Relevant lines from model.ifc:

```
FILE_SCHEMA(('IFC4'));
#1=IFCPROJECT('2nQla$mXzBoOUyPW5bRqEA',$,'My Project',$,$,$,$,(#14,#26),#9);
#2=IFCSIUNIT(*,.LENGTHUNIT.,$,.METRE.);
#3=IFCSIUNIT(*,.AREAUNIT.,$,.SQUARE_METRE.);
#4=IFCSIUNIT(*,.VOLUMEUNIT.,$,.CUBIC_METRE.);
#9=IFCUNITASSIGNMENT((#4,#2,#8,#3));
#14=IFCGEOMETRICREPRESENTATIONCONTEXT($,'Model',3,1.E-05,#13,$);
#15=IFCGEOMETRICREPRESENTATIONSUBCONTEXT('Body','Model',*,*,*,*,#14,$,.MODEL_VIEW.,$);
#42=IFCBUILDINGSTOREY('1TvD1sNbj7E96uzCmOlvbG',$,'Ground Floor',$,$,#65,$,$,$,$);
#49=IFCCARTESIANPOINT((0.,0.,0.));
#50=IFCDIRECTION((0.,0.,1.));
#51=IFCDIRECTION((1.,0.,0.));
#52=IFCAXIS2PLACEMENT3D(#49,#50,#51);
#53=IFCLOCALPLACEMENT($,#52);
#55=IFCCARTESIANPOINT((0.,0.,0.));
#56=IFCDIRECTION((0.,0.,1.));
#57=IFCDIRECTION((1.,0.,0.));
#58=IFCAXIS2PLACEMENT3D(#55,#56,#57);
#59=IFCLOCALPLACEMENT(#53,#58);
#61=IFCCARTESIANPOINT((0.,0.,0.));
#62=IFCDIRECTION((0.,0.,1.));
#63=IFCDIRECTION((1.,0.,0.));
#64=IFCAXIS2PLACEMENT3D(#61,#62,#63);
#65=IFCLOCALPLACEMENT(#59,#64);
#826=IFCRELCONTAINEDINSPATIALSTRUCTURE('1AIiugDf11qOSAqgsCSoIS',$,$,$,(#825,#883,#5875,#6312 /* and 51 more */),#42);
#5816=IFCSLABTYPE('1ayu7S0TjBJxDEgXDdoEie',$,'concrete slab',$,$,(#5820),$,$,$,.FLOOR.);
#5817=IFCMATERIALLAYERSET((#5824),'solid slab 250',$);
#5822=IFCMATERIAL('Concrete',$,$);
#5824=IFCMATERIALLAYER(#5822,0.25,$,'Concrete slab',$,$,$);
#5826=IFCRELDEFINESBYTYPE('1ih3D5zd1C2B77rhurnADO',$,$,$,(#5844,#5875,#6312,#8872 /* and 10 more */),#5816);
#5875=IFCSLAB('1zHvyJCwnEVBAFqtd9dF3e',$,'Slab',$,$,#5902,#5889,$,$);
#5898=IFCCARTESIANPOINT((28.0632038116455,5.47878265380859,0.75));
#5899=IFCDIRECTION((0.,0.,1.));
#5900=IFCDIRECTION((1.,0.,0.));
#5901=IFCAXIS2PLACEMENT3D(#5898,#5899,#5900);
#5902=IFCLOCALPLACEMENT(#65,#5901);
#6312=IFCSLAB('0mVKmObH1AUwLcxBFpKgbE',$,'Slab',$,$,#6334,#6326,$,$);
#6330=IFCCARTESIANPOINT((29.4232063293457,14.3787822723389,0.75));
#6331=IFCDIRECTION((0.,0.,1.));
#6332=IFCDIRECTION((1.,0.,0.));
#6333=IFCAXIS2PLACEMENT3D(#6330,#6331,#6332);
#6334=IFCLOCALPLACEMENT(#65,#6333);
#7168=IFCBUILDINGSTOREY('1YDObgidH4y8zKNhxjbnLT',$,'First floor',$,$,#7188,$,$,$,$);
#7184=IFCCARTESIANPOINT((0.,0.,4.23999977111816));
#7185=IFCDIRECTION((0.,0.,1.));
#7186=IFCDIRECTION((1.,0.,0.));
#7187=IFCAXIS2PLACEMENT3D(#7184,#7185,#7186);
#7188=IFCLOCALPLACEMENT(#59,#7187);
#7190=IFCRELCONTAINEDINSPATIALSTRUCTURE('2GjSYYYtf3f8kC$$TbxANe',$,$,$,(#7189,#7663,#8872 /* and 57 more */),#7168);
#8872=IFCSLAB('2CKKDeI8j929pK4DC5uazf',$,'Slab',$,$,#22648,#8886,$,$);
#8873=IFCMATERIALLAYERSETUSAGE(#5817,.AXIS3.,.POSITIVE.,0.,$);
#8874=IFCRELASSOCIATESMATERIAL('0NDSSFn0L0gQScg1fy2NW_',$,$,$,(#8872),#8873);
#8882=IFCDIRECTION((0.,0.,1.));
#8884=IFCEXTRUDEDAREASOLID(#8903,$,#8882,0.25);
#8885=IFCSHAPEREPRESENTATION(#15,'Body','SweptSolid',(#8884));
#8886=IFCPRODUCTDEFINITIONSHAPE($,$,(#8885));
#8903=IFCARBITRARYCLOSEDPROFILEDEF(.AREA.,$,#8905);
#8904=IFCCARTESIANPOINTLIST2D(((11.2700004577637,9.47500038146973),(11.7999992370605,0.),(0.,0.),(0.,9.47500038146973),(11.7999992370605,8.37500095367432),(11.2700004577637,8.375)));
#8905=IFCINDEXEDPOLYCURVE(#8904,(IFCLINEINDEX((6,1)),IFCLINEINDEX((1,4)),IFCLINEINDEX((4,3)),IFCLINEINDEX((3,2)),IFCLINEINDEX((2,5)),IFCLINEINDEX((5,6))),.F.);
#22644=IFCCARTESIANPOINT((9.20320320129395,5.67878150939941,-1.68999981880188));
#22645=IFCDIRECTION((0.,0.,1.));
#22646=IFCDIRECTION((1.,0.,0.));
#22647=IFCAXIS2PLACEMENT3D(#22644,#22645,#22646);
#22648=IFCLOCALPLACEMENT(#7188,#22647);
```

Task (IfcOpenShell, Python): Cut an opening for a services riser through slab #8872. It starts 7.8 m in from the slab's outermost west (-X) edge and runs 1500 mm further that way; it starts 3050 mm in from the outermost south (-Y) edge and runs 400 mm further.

```python
import numpy as np
import ifcopenshell
import ifcopenshell.api.feature
import ifcopenshell.api.geometry
import ifcopenshell.api.root
import ifcopenshell.geom
import ifcopenshell.util.placement
import ifcopenshell.util.representation
import ifcopenshell.util.shape
import ifcopenshell.util.unit

model = ifcopenshell.open("model.ifc")
unit_scale = ifcopenshell.util.unit.calculate_unit_scale(model)
settings = ifcopenshell.geom.settings()


def volume(element):
    """Net volume in cubic metres, openings subtracted."""
    shape = ifcopenshell.geom.create_shape(settings, element)
    return ifcopenshell.util.shape.get_volume(shape.geometry)


slab = model.by_guid("2CKKDeI8j929pK4DC5uazf")
before = volume(slab)

# Extent in the slab's own axes, in metres. The edges named are its -X and -Y sides.
slab_shape = ifcopenshell.geom.create_shape(settings, slab)
vertices = ifcopenshell.util.shape.get_vertices(slab_shape.geometry)
x_min, y_min, bottom = vertices.min(axis=0)
top = vertices[:, 2].max()

opening = ifcopenshell.api.root.create_entity(model, ifc_class="IfcOpeningElement", name="Services riser opening", predefined_type="OPENING")
context = ifcopenshell.util.representation.get_context(model, "Model", "Body", "MODEL_VIEW")
width, depth = 1.5, 0.4
outline = [(0.0, 0.0), (width, 0.0), (width, depth), (0.0, depth), (0.0, 0.0)]
# Overshoot both faces by 50 mm so the cut is clean.
shape = ifcopenshell.api.geometry.add_slab_representation(
    model, context=context, depth=top - bottom + 0.1, polyline=outline
)
ifcopenshell.api.geometry.assign_representation(model, product=opening, representation=shape)

matrix = ifcopenshell.util.placement.get_local_placement(slab.ObjectPlacement)
matrix[:, 3] = matrix @ np.append(np.array([x_min + 7.8, y_min + 3.05, bottom - 0.05]) / unit_scale, 1.0)
ifcopenshell.api.geometry.edit_object_placement(model, product=opening, matrix=matrix, is_si=False)
ifcopenshell.api.feature.add_feature(model, feature=opening, element=slab)

after = volume(slab)

print(f"slab volume {before:.3f} -> {after:.3f} m3")

model.write("model_edited.ifc")
```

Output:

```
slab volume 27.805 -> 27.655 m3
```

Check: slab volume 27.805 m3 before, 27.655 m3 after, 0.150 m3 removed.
